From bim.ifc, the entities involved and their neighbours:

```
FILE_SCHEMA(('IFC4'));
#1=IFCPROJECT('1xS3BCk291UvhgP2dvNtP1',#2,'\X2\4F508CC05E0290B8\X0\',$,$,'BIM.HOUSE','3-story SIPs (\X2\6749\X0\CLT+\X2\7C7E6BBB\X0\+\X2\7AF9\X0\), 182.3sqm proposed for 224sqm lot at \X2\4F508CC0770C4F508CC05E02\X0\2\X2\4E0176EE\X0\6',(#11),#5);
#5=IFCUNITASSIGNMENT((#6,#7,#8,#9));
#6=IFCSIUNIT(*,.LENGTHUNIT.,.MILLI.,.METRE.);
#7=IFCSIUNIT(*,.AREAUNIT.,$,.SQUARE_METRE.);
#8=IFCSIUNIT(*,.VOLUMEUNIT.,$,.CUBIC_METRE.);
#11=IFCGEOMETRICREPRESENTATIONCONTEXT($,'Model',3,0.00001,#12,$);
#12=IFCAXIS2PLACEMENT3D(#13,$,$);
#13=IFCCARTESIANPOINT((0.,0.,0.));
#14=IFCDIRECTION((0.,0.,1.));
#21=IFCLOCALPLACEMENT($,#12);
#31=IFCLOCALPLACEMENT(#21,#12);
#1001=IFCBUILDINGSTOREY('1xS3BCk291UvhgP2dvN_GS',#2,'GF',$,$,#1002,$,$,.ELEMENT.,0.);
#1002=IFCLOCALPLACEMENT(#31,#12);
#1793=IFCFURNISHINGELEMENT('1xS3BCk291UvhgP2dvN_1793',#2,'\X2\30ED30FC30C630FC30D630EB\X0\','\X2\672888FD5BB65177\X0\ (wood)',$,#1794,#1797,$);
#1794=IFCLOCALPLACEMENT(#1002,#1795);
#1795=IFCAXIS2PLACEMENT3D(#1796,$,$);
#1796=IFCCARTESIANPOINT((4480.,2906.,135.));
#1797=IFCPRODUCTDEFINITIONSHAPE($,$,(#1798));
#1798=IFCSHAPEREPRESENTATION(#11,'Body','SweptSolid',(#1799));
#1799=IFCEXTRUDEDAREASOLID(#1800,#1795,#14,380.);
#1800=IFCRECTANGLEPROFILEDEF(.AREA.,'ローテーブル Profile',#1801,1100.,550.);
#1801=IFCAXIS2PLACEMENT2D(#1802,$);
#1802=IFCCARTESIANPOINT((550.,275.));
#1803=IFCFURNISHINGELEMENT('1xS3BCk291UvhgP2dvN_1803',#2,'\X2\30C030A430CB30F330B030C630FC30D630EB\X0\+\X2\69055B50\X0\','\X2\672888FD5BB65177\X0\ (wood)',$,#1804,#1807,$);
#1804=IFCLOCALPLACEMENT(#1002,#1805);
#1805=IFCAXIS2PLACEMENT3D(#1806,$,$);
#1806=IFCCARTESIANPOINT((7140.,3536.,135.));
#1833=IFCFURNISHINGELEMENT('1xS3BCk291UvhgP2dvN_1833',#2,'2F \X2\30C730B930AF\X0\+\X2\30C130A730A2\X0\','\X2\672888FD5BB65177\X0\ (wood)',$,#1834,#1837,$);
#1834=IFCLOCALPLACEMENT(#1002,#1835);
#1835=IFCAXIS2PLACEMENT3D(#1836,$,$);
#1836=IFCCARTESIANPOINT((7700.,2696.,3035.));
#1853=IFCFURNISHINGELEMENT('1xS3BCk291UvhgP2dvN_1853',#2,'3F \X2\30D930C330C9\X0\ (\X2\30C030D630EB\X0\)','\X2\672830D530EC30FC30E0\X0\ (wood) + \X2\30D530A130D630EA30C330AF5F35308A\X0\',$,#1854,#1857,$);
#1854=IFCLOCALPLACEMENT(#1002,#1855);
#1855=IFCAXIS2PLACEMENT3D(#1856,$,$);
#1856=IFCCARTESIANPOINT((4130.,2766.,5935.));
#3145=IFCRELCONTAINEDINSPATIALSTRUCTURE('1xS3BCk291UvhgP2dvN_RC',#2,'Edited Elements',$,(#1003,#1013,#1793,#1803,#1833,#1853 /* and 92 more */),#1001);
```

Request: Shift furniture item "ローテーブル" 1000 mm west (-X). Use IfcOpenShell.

```python
import ifcopenshell
import ifcopenshell.api.geometry
import ifcopenshell.util.placement

model = ifcopenshell.open("bim.ifc")

item = model.by_guid("1xS3BCk291UvhgP2dvN_1793")
matrix = ifcopenshell.util.placement.get_local_placement(item.ObjectPlacement)
matrix[0, 3] -= 1000.0
ifcopenshell.api.geometry.edit_object_placement(model, product=item, matrix=matrix, is_si=False)

print(ifcopenshell.util.placement.get_local_placement(item.ObjectPlacement).round(3) + 0.0)

model.write("bim_rev.ifc")
```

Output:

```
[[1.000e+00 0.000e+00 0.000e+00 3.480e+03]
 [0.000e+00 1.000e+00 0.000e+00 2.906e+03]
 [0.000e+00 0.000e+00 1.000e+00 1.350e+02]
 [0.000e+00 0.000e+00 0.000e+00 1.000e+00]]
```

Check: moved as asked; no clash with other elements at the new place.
